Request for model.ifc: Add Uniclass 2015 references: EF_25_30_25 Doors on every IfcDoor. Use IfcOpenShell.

First a look at what the model holds.

```python
import ifcopenshell

model = ifcopenshell.open("model.ifc")
print(model.schema)
print("classifications:", [c.Name for c in model.by_type("IfcClassification")])
for ifc_class in ("IfcDoor", "IfcRoof", "IfcStair", "IfcWall", "IfcWindow"):
    print(ifc_class, len(model.by_type(ifc_class)))
```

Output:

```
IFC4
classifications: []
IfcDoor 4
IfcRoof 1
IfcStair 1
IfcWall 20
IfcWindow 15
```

```python
import ifcopenshell
import ifcopenshell.api.classification

model = ifcopenshell.open("model.ifc")

system = ifcopenshell.api.classification.add_classification(model, classification="Uniclass 2015")

codes = {
    "IfcDoor": ("EF_25_30_25", "Doors"),
}
for ifc_class, (code, name) in codes.items():
    products = model.by_type(ifc_class)
    ifcopenshell.api.classification.add_reference(
        model, products=products, classification=system, identification=code, name=name
    )
    print(code, len(products))

model.write("model_updated.ifc")
```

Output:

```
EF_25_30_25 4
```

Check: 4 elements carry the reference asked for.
